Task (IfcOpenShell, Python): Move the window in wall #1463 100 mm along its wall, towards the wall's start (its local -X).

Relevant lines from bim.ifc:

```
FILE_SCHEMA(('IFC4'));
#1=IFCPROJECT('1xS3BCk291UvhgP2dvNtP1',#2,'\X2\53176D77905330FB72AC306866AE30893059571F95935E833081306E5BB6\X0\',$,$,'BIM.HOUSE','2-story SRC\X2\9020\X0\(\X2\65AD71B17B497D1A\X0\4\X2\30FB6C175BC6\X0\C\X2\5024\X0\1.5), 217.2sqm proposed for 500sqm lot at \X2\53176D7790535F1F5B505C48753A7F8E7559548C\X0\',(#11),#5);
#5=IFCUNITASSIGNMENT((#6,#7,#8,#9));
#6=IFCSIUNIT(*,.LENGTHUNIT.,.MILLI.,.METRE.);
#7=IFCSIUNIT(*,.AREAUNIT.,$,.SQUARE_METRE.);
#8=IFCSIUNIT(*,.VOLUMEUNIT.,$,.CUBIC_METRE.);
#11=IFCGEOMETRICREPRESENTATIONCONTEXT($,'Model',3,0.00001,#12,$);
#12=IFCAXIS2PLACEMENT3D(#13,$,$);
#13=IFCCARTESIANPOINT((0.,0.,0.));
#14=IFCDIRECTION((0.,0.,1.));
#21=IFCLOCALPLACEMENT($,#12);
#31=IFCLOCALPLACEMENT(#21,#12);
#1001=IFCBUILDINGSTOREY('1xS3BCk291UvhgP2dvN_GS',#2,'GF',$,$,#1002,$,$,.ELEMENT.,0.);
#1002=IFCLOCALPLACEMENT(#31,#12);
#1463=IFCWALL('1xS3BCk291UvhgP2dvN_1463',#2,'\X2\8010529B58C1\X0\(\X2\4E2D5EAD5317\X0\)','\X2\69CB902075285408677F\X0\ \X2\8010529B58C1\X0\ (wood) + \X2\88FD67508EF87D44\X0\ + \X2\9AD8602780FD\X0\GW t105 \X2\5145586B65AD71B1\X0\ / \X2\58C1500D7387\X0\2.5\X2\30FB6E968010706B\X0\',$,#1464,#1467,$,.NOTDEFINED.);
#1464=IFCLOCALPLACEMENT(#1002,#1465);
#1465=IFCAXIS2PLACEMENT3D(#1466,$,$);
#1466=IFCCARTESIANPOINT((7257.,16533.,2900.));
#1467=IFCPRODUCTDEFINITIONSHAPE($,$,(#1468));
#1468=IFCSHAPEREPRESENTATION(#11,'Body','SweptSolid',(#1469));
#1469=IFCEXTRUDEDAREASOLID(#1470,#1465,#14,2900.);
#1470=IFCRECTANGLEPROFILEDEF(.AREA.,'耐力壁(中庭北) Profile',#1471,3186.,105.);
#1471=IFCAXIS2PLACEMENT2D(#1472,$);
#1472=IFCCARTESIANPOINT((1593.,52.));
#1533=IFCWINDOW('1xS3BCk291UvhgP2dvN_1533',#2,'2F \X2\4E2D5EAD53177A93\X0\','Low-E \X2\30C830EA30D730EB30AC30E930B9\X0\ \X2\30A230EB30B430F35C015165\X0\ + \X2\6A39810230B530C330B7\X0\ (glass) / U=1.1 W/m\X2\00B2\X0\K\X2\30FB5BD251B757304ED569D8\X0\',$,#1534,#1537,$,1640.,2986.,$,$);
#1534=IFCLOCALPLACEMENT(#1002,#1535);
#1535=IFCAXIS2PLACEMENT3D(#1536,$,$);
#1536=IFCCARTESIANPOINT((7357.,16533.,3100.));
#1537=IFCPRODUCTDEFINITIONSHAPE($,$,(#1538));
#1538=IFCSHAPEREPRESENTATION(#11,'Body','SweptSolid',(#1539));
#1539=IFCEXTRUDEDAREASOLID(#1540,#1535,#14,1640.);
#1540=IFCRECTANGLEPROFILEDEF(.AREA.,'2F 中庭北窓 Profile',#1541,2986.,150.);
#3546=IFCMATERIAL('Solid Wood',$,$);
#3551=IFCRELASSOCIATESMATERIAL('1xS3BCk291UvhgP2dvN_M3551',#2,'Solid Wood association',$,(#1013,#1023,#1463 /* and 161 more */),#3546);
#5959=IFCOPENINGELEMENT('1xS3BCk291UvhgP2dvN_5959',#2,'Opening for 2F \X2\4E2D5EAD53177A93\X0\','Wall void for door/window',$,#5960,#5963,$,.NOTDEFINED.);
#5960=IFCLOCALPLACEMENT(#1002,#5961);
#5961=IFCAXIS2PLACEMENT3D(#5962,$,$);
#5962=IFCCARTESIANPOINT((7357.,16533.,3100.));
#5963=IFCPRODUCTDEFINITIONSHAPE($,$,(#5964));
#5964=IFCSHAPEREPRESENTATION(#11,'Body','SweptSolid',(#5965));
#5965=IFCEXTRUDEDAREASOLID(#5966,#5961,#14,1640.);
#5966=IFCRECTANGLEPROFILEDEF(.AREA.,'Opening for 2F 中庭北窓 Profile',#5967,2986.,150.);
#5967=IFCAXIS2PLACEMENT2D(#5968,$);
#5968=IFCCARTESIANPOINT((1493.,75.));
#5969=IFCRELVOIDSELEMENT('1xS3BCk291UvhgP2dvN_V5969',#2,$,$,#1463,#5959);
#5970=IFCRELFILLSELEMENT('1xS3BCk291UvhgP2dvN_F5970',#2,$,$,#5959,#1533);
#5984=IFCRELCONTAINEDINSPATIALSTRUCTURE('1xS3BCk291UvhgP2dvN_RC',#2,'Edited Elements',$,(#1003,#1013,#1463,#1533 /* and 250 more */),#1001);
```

```python
import ifcopenshell
import ifcopenshell.api.geometry
import ifcopenshell.util.placement
import ifcopenshell.util.unit

model = ifcopenshell.open("bim.ifc")
unit_scale = ifcopenshell.util.unit.calculate_unit_scale(model)

window = model.by_id(1533)
opening = window.FillsVoids[0].RelatingOpeningElement
wall = opening.VoidsElements[0].RelatingBuildingElement

wall_matrix = ifcopenshell.util.placement.get_local_placement(wall.ObjectPlacement)
shift = wall_matrix[:3, 0] * -0.1 / unit_scale
before = ifcopenshell.util.placement.get_local_placement(window.ObjectPlacement)[:3, 3].copy()

# The window is not placed relative to its opening, so move both.
for product in (opening, window):
    matrix = ifcopenshell.util.placement.get_local_placement(product.ObjectPlacement)
    matrix[:3, 3] += shift
    ifcopenshell.api.geometry.edit_object_placement(model, product=product, matrix=matrix, is_si=False)

after = ifcopenshell.util.placement.get_local_placement(window.ObjectPlacement)[:3, 3]
print("window moved by", (after - before).round(3) + 0.0)

model.write("bim-out.ifc")
```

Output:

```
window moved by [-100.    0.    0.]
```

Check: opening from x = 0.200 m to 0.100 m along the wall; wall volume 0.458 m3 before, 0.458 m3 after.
